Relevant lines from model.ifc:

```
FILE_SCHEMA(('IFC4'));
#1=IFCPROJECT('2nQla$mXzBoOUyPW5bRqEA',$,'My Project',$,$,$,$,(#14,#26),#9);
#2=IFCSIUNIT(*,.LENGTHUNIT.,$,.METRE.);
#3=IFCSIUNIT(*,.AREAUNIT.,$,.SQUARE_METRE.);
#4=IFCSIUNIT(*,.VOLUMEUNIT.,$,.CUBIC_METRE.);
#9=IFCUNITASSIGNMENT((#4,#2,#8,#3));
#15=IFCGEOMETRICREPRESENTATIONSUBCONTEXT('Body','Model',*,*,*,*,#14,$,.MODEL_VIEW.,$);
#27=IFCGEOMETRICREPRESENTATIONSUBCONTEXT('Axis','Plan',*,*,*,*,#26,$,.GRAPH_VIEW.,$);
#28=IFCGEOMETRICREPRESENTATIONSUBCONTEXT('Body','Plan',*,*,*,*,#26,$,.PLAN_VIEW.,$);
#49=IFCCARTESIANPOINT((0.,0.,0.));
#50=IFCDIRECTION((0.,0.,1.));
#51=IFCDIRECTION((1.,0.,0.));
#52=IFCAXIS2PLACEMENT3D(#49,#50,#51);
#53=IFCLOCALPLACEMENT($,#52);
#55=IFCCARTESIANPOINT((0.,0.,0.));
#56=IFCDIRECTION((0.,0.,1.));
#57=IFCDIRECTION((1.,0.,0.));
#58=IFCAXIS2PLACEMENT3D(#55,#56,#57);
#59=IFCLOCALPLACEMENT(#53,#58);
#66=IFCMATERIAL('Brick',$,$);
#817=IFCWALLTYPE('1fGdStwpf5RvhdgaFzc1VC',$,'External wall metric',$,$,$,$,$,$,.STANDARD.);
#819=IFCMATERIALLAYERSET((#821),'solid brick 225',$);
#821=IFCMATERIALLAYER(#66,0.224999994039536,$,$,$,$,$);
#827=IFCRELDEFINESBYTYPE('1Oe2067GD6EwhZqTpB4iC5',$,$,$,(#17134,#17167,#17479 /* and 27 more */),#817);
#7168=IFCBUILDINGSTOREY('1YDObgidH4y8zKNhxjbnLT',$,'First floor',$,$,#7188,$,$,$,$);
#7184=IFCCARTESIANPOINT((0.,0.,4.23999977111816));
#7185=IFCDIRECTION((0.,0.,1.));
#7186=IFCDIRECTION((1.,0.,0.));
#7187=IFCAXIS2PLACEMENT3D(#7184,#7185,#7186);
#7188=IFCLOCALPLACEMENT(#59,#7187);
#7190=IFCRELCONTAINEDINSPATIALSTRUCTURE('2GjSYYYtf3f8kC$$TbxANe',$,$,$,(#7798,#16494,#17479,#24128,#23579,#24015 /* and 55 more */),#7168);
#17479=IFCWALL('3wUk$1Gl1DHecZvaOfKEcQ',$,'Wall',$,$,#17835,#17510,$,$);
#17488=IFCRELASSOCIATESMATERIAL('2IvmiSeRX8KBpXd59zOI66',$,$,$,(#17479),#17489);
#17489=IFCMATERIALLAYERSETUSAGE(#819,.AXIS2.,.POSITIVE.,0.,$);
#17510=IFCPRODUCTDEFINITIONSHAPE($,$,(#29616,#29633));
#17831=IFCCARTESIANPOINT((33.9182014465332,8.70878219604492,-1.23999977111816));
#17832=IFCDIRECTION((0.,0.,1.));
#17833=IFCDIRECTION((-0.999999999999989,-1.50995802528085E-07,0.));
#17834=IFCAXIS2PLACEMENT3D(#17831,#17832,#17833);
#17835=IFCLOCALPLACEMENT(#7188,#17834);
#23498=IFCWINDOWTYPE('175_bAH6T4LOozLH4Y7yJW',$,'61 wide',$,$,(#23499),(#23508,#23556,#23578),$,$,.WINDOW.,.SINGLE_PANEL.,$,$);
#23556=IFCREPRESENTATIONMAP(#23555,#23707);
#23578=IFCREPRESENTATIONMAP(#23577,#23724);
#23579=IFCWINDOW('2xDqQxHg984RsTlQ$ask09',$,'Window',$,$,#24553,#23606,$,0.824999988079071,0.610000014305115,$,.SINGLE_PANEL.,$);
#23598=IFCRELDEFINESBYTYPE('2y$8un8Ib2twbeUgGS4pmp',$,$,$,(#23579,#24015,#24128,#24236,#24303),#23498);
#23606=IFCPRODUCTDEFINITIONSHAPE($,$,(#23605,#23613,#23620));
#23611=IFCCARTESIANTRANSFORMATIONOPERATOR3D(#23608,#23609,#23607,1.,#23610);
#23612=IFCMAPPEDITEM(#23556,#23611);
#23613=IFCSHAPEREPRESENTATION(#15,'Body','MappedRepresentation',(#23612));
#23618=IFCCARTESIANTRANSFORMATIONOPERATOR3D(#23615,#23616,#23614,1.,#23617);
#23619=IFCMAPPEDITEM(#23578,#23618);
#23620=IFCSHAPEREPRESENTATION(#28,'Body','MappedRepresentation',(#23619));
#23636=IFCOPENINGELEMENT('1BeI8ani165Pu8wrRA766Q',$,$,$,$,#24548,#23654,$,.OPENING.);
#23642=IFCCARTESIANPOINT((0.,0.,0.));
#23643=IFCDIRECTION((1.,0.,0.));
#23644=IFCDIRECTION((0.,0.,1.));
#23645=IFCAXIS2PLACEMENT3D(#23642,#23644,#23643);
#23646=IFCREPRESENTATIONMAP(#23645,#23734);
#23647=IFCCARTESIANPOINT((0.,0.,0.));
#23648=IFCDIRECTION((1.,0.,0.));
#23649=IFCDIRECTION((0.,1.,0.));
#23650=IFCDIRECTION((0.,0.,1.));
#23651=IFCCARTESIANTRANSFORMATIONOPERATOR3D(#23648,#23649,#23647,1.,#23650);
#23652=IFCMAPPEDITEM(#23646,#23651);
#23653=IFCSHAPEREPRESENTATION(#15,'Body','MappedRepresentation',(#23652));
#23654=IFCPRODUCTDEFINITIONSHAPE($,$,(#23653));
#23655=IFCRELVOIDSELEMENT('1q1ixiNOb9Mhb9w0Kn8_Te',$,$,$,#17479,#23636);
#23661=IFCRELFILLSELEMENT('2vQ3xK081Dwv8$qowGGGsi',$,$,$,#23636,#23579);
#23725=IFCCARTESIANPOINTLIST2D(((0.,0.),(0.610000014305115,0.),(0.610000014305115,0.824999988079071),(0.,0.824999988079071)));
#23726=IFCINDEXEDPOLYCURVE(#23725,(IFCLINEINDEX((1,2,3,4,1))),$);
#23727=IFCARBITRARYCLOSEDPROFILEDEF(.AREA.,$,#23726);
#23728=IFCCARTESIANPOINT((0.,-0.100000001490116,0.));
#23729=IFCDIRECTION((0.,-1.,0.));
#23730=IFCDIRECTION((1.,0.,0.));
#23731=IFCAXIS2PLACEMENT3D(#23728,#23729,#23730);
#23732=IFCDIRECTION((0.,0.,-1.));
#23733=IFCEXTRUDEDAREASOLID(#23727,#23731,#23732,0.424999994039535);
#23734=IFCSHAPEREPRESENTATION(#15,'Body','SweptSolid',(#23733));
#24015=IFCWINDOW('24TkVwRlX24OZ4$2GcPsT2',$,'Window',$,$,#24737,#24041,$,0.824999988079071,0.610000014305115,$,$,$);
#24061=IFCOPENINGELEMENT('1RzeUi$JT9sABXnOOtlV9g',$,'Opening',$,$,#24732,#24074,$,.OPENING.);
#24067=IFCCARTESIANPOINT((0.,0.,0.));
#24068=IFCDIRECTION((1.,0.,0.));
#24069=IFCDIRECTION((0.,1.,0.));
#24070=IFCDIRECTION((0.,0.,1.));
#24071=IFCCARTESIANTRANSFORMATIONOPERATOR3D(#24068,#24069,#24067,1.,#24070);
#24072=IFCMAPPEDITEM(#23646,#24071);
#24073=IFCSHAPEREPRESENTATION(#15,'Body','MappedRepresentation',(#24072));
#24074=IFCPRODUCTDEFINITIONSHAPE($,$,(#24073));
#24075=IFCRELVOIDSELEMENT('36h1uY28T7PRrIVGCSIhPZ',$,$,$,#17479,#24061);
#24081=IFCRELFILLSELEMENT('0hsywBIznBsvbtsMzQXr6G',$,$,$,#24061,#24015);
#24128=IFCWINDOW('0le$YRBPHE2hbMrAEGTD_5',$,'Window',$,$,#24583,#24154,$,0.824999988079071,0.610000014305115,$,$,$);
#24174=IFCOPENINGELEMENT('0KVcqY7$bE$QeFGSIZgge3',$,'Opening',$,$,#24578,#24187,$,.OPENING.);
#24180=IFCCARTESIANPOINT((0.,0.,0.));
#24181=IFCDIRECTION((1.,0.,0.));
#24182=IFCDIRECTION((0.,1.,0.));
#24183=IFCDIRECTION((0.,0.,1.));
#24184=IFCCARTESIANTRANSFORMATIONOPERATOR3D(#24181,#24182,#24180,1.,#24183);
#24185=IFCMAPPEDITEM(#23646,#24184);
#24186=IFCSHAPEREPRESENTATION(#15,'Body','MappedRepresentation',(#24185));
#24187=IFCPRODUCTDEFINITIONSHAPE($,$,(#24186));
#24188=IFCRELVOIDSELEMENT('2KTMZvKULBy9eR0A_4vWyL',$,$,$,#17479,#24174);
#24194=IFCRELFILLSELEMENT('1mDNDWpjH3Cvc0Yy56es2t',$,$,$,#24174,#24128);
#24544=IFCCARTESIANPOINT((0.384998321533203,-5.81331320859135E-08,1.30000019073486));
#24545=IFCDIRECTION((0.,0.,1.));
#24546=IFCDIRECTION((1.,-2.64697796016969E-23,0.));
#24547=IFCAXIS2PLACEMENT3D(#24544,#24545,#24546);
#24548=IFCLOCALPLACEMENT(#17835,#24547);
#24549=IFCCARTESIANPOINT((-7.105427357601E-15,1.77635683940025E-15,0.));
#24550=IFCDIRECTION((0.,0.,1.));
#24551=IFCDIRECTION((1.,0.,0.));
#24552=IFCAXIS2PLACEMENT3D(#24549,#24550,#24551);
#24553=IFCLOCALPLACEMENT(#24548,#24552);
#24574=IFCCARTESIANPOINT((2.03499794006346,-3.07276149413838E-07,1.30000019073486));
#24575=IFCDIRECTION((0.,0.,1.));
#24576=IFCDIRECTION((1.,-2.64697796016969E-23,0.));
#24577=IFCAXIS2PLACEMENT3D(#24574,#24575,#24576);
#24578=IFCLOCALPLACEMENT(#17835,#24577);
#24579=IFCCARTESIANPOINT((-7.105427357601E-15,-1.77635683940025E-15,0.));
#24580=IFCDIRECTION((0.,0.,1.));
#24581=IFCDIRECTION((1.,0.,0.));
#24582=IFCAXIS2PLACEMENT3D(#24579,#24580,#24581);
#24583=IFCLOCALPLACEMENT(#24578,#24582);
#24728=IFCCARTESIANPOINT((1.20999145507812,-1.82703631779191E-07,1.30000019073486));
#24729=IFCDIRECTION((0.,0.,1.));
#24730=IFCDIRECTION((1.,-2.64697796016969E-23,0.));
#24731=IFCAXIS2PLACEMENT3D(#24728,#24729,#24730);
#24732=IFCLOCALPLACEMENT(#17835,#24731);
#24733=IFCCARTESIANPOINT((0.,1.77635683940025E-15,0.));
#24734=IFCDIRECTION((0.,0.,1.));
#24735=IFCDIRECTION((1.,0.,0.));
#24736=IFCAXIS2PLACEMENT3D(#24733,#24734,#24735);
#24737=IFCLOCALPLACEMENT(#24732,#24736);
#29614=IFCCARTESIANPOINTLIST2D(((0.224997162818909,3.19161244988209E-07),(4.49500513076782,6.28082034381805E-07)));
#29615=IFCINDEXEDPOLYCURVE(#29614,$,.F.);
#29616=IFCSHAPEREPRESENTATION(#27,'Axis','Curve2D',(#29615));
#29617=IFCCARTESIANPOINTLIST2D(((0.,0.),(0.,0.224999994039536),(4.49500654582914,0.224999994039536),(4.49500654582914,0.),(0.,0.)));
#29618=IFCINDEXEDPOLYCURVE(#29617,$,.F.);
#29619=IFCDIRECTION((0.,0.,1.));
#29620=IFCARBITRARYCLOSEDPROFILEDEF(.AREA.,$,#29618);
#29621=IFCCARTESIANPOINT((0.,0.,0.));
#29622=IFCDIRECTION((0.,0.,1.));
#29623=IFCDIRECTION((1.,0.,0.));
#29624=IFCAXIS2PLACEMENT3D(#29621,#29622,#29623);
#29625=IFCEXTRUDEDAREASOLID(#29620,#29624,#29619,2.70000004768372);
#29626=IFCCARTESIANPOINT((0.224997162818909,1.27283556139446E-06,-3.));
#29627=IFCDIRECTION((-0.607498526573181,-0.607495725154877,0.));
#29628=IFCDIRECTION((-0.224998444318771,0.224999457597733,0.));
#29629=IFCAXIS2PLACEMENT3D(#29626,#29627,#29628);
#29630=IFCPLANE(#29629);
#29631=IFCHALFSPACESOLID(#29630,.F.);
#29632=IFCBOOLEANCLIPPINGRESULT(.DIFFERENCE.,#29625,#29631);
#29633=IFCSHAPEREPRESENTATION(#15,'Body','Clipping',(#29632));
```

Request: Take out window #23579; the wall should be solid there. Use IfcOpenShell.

```python
import ifcopenshell
import ifcopenshell.api.feature
import ifcopenshell.api.root
import ifcopenshell.geom
import ifcopenshell.util.shape

model = ifcopenshell.open("model.ifc")
settings = ifcopenshell.geom.settings()


def volume(element):
    """Net volume in cubic metres, openings subtracted."""
    shape = ifcopenshell.geom.create_shape(settings, element)
    return ifcopenshell.util.shape.get_volume(shape.geometry)


window = model.by_guid("2xDqQxHg984RsTlQ$ask09")
opening = window.FillsVoids[0].RelatingOpeningElement
wall = opening.VoidsElements[0].RelatingBuildingElement
before = volume(wall)

ifcopenshell.api.root.remove_product(model, product=window)
ifcopenshell.api.feature.remove_feature(model, feature=opening)

after = volume(wall)

print(f"wall volume {before:.3f} -> {after:.3f} m3")

model.write("model_updated.ifc")
```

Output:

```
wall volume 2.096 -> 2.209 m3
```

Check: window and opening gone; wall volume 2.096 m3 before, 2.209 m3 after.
